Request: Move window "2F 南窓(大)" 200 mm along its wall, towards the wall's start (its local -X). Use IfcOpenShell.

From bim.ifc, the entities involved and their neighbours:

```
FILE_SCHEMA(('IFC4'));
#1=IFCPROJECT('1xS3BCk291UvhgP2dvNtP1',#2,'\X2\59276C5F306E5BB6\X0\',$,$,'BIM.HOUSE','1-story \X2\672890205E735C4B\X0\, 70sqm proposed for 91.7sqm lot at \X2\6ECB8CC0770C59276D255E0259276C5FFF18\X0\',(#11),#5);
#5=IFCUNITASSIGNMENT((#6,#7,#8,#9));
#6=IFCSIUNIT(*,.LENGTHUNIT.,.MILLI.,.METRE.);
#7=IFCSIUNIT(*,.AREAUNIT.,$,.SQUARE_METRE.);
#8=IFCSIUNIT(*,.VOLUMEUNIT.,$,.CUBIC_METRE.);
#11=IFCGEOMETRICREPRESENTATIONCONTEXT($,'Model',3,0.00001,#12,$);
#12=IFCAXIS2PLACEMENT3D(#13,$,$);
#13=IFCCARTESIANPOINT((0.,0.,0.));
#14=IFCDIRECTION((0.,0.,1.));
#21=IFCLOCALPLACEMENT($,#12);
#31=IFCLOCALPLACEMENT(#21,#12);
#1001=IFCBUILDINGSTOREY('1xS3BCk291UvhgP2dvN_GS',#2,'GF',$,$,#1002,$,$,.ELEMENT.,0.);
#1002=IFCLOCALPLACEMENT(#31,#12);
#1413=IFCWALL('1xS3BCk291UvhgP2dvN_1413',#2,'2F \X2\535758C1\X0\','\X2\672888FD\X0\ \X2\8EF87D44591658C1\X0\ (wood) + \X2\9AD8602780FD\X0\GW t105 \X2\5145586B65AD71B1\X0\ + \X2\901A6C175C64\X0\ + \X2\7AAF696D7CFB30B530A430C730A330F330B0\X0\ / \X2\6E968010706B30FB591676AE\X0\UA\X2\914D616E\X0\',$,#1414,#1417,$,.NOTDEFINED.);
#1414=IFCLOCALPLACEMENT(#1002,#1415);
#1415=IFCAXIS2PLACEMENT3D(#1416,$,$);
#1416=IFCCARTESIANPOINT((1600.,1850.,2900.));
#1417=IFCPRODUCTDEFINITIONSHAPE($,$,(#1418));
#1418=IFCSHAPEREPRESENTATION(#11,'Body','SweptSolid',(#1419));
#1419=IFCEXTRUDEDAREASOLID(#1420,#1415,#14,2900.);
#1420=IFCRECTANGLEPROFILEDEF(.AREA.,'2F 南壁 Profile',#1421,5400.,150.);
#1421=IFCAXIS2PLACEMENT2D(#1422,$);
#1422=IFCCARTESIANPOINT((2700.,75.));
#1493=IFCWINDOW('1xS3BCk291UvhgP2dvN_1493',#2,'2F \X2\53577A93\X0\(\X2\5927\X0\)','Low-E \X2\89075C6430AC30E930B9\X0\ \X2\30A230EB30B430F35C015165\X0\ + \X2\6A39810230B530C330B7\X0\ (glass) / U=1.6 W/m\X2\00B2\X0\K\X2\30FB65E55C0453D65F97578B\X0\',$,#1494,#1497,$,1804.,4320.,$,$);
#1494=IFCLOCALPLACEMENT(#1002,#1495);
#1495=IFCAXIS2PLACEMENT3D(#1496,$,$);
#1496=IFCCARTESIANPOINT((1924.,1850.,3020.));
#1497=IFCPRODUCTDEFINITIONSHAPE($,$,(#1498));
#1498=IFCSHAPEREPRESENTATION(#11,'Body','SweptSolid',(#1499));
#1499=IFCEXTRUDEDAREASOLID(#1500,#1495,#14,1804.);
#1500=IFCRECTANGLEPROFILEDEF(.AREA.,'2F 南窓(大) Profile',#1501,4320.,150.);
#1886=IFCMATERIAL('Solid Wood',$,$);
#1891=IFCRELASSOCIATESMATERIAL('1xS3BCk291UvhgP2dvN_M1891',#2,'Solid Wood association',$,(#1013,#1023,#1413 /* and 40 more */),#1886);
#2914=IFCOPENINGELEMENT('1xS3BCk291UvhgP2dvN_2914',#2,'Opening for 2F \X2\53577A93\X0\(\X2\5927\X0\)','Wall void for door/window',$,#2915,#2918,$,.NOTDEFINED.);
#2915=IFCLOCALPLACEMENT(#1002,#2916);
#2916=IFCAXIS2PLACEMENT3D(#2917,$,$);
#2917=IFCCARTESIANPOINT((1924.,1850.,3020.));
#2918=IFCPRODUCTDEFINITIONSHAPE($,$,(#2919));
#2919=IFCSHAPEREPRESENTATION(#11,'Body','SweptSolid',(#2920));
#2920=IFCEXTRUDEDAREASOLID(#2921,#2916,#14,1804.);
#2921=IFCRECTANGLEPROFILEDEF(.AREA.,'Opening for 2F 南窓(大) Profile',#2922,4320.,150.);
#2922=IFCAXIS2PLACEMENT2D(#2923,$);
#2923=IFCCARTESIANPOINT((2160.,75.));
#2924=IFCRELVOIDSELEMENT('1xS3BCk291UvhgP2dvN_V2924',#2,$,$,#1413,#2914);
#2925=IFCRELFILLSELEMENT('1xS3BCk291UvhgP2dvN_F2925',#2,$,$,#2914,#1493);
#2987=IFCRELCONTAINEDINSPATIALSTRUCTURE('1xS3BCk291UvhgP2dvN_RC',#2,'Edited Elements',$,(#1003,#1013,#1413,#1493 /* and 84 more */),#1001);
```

```python
import ifcopenshell
import ifcopenshell.api.geometry
import ifcopenshell.util.placement

model = ifcopenshell.open("bim.ifc")

window = model.by_guid("1xS3BCk291UvhgP2dvN_1493")
opening = window.FillsVoids[0].RelatingOpeningElement
wall = opening.VoidsElements[0].RelatingBuildingElement

wall_matrix = ifcopenshell.util.placement.get_local_placement(wall.ObjectPlacement)
shift = wall_matrix[:3, 0] * -200.0
before = ifcopenshell.util.placement.get_local_placement(window.ObjectPlacement)[:3, 3].copy()

# The window is not placed relative to its opening, so move both.
for product in (opening, window):
    matrix = ifcopenshell.util.placement.get_local_placement(product.ObjectPlacement)
    matrix[:3, 3] += shift
    ifcopenshell.api.geometry.edit_object_placement(model, product=product, matrix=matrix, is_si=False)

after = ifcopenshell.util.placement.get_local_placement(window.ObjectPlacement)[:3, 3]
print("window moved by", (after - before).round(3) + 0.0)

model.write("bim_rev.ifc")
```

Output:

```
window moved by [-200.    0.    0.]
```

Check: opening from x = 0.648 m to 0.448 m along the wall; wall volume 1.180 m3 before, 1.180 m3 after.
